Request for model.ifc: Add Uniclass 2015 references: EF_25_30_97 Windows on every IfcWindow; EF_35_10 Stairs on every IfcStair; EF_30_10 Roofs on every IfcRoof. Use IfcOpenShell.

First a look at what the model holds.

```python
import ifcopenshell

model = ifcopenshell.open("model.ifc")
print(model.schema)
print("classifications:", [c.Name for c in model.by_type("IfcClassification")])
for ifc_class in ("IfcDoor", "IfcRoof", "IfcStair", "IfcWall", "IfcWindow"):
    print(ifc_class, len(model.by_type(ifc_class)))
```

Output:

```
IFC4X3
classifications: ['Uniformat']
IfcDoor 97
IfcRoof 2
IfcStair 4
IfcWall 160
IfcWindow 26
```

```python
import ifcopenshell
import ifcopenshell.api.classification

model = ifcopenshell.open("model.ifc")

system = ifcopenshell.api.classification.add_classification(model, classification="Uniclass 2015")

codes = {
    "IfcWindow": ("EF_25_30_97", "Windows"),
    "IfcStair": ("EF_35_10", "Stairs"),
    "IfcRoof": ("EF_30_10", "Roofs"),
}
for ifc_class, (code, name) in codes.items():
    products = model.by_type(ifc_class)
    ifcopenshell.api.classification.add_reference(
        model, products=products, classification=system, identification=code, name=name
    )
    print(code, len(products))

model.write("model_rev.ifc")
```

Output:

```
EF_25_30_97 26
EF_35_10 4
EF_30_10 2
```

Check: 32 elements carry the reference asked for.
